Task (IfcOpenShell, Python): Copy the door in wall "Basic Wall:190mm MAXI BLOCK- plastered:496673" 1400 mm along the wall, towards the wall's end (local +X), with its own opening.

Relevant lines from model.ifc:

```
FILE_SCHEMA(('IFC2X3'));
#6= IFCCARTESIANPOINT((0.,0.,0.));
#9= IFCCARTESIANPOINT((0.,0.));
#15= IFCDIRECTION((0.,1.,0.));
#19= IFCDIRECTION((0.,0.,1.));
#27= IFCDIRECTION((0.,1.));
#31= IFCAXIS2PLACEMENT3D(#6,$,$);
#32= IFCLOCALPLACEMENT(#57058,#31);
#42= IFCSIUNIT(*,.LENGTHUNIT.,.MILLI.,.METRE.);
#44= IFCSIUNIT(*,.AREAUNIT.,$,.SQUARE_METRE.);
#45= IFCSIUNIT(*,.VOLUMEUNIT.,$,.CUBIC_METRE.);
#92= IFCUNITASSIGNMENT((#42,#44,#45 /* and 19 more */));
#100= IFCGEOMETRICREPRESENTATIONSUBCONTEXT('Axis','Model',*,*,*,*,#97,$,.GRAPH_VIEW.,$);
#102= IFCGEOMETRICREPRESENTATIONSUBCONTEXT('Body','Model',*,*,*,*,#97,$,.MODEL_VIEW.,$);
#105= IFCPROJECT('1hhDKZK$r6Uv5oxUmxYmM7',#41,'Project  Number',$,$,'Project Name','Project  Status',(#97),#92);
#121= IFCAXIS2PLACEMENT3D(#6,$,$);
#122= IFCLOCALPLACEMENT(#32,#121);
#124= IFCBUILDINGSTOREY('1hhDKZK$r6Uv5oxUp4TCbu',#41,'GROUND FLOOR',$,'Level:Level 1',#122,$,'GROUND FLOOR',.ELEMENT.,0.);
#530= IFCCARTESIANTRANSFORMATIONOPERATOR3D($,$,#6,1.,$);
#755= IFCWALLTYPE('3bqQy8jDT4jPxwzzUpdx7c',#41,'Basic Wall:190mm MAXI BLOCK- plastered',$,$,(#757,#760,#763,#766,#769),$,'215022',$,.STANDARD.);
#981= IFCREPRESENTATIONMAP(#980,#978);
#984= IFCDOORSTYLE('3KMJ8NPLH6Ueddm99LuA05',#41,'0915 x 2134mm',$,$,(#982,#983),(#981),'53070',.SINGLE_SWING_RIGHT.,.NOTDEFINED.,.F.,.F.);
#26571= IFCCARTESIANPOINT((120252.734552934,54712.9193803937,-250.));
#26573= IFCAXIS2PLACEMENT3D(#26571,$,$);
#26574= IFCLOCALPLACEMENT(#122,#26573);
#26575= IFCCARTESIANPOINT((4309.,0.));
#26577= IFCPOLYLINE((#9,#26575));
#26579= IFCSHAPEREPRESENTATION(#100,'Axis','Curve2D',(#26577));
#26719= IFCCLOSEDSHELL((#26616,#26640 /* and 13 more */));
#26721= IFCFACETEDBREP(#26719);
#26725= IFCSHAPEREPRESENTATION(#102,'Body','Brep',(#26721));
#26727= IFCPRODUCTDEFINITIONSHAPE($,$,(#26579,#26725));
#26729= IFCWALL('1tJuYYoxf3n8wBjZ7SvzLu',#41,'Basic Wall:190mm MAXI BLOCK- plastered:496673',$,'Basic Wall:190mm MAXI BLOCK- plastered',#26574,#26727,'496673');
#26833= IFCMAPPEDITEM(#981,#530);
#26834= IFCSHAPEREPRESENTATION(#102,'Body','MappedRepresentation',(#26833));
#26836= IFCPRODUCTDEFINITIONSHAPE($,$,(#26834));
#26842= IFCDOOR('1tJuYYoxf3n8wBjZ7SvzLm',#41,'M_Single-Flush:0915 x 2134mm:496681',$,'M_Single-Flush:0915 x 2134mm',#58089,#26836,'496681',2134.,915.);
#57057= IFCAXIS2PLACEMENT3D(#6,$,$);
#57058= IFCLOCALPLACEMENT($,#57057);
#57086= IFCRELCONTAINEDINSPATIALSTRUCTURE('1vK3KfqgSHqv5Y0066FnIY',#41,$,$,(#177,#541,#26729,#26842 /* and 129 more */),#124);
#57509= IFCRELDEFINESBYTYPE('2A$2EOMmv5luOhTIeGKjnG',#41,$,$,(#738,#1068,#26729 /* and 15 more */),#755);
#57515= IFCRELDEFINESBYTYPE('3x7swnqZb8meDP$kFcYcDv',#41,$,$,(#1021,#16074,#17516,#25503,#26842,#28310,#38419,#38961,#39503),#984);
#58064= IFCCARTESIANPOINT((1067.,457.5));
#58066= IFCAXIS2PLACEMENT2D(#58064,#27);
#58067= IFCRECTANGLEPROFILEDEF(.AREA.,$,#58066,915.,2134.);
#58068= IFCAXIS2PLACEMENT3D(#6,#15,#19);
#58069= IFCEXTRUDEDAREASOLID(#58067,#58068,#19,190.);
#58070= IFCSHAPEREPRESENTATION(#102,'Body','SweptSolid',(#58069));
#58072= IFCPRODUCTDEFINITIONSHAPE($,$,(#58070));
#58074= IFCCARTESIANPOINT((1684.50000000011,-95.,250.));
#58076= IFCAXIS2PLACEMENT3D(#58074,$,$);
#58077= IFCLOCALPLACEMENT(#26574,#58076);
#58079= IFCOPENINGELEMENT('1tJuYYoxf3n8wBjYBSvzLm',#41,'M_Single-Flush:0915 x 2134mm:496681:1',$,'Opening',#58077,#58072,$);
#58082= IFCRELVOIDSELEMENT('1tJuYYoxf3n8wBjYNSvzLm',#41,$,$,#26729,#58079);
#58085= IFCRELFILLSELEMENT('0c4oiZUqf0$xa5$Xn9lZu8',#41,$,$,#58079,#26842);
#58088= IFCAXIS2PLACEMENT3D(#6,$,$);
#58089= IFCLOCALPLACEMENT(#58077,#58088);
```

```python
import ifcopenshell
import ifcopenshell.api.feature
import ifcopenshell.api.geometry
import ifcopenshell.api.root
import ifcopenshell.geom
import ifcopenshell.util.element
import ifcopenshell.util.placement
import ifcopenshell.util.shape
import ifcopenshell.util.unit

model = ifcopenshell.open("model.ifc")
unit_scale = ifcopenshell.util.unit.calculate_unit_scale(model)
settings = ifcopenshell.geom.settings()


def volume(element):
    """Net volume in cubic metres, openings subtracted."""
    shape = ifcopenshell.geom.create_shape(settings, element)
    return ifcopenshell.util.shape.get_volume(shape.geometry)


def reuse_history(source, copy):
    """copy_class also copies each property set's owner history, people and application; keep the originals."""
    for rel in copy.IsDefinedBy:
        if rel.is_a("IfcRelDefinesByProperties") and (history := rel.RelatingPropertyDefinition.OwnerHistory):
            rel.RelatingPropertyDefinition.OwnerHistory = source.OwnerHistory
            ifcopenshell.util.element.remove_deep2(model, history)


door = model.by_id(26842)
opening = door.FillsVoids[0].RelatingOpeningElement
wall = opening.VoidsElements[0].RelatingBuildingElement
before = volume(wall)
shift = ifcopenshell.util.placement.get_local_placement(wall.ObjectPlacement)[:3, 0] * 1.4 / unit_scale

# copy_class copies the void relationship, type, container and properties, but no geometry.
new_opening = ifcopenshell.api.root.copy_class(model, product=opening)
new_opening.Representation = ifcopenshell.util.element.copy_deep(
    model, opening.Representation, exclude=["IfcGeometricRepresentationContext", "IfcRepresentationMap"]
)
new_opening.Name = "M_Single-Flush:0915 x 2134mm"
new_door = ifcopenshell.api.root.copy_class(model, product=door)
new_door.Representation = ifcopenshell.util.element.copy_deep(
    model, door.Representation, exclude=["IfcGeometricRepresentationContext", "IfcRepresentationMap"]
)
new_door.Name = "M_Single-Flush:0915 x 2134mm"
new_door.Tag = None
reuse_history(door, new_door)
fills = ifcopenshell.api.feature.add_filling(model, opening=new_opening, element=new_door)
fills.OwnerHistory = new_door.OwnerHistory  # required in IFC2X3

for old, new in ((opening, new_opening), (door, new_door)):
    matrix = ifcopenshell.util.placement.get_local_placement(old.ObjectPlacement)
    matrix[:3, 3] += shift
    ifcopenshell.api.geometry.edit_object_placement(model, product=new, matrix=matrix, is_si=False)

after = volume(wall)

print(f"wall volume {before:.3f} -> {after:.3f} m3")

model.write("model_edited.ifc")
```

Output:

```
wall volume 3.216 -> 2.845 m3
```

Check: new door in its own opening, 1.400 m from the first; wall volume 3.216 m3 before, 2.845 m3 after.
